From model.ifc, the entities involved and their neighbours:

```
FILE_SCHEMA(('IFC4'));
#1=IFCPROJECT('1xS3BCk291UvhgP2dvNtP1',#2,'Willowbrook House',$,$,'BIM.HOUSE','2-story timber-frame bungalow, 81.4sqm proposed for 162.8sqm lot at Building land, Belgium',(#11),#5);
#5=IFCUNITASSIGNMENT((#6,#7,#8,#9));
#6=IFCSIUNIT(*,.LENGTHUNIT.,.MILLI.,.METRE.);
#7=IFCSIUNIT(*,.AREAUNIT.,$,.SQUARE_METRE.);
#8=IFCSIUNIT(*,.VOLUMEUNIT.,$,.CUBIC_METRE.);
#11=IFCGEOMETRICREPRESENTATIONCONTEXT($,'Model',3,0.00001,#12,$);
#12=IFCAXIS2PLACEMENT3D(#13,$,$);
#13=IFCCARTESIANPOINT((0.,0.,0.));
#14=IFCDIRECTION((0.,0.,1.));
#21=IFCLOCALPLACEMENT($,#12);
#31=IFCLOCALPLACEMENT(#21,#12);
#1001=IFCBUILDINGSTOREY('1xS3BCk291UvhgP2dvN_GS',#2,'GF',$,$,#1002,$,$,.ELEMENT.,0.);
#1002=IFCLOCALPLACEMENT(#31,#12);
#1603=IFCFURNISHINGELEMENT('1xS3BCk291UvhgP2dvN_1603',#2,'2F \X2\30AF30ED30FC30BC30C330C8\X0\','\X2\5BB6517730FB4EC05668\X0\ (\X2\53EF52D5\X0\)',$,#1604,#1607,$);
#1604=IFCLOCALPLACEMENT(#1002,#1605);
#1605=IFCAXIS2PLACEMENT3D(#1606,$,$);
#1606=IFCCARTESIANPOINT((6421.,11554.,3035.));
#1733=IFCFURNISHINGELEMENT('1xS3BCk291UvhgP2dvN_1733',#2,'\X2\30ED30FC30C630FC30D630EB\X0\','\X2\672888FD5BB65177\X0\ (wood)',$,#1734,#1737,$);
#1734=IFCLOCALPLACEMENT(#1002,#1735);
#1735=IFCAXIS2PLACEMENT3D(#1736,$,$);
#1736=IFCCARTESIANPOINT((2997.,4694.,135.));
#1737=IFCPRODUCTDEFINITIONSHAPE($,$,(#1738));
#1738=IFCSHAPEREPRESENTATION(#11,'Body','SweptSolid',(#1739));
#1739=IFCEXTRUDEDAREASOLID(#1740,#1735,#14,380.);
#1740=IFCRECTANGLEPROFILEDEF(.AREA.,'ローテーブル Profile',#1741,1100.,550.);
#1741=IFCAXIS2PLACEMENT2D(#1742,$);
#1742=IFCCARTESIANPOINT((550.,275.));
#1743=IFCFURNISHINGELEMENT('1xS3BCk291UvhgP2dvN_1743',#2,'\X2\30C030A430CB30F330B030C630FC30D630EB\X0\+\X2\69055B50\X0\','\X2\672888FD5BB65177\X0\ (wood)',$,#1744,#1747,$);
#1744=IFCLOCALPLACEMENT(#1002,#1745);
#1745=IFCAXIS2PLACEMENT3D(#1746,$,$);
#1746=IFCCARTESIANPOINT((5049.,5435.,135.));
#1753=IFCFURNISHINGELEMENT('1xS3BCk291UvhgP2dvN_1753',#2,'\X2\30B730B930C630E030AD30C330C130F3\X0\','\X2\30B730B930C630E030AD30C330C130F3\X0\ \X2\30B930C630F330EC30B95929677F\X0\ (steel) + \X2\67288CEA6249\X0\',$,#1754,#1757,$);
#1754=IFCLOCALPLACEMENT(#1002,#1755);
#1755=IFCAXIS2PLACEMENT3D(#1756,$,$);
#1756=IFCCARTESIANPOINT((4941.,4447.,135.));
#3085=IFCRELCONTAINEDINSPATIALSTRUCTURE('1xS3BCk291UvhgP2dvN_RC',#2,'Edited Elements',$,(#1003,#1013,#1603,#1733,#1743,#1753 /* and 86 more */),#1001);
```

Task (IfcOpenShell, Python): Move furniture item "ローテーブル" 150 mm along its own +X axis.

```python
import ifcopenshell
import ifcopenshell.api.geometry
import ifcopenshell.util.placement
import ifcopenshell.util.unit

model = ifcopenshell.open("model.ifc")
unit_scale = ifcopenshell.util.unit.calculate_unit_scale(model)

item = model.by_guid("1xS3BCk291UvhgP2dvN_1733")
matrix = ifcopenshell.util.placement.get_local_placement(item.ObjectPlacement)
matrix[:3, 3] += matrix[:3, 0] * 0.15 / unit_scale
ifcopenshell.api.geometry.edit_object_placement(model, product=item, matrix=matrix, is_si=False)

print(ifcopenshell.util.placement.get_local_placement(item.ObjectPlacement).round(3) + 0.0)

model.write("model_rev.ifc")
```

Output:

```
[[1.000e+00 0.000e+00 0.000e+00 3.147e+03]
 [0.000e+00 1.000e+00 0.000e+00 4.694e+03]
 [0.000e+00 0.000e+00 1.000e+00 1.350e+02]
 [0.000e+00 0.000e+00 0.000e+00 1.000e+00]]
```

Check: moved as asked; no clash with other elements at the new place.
